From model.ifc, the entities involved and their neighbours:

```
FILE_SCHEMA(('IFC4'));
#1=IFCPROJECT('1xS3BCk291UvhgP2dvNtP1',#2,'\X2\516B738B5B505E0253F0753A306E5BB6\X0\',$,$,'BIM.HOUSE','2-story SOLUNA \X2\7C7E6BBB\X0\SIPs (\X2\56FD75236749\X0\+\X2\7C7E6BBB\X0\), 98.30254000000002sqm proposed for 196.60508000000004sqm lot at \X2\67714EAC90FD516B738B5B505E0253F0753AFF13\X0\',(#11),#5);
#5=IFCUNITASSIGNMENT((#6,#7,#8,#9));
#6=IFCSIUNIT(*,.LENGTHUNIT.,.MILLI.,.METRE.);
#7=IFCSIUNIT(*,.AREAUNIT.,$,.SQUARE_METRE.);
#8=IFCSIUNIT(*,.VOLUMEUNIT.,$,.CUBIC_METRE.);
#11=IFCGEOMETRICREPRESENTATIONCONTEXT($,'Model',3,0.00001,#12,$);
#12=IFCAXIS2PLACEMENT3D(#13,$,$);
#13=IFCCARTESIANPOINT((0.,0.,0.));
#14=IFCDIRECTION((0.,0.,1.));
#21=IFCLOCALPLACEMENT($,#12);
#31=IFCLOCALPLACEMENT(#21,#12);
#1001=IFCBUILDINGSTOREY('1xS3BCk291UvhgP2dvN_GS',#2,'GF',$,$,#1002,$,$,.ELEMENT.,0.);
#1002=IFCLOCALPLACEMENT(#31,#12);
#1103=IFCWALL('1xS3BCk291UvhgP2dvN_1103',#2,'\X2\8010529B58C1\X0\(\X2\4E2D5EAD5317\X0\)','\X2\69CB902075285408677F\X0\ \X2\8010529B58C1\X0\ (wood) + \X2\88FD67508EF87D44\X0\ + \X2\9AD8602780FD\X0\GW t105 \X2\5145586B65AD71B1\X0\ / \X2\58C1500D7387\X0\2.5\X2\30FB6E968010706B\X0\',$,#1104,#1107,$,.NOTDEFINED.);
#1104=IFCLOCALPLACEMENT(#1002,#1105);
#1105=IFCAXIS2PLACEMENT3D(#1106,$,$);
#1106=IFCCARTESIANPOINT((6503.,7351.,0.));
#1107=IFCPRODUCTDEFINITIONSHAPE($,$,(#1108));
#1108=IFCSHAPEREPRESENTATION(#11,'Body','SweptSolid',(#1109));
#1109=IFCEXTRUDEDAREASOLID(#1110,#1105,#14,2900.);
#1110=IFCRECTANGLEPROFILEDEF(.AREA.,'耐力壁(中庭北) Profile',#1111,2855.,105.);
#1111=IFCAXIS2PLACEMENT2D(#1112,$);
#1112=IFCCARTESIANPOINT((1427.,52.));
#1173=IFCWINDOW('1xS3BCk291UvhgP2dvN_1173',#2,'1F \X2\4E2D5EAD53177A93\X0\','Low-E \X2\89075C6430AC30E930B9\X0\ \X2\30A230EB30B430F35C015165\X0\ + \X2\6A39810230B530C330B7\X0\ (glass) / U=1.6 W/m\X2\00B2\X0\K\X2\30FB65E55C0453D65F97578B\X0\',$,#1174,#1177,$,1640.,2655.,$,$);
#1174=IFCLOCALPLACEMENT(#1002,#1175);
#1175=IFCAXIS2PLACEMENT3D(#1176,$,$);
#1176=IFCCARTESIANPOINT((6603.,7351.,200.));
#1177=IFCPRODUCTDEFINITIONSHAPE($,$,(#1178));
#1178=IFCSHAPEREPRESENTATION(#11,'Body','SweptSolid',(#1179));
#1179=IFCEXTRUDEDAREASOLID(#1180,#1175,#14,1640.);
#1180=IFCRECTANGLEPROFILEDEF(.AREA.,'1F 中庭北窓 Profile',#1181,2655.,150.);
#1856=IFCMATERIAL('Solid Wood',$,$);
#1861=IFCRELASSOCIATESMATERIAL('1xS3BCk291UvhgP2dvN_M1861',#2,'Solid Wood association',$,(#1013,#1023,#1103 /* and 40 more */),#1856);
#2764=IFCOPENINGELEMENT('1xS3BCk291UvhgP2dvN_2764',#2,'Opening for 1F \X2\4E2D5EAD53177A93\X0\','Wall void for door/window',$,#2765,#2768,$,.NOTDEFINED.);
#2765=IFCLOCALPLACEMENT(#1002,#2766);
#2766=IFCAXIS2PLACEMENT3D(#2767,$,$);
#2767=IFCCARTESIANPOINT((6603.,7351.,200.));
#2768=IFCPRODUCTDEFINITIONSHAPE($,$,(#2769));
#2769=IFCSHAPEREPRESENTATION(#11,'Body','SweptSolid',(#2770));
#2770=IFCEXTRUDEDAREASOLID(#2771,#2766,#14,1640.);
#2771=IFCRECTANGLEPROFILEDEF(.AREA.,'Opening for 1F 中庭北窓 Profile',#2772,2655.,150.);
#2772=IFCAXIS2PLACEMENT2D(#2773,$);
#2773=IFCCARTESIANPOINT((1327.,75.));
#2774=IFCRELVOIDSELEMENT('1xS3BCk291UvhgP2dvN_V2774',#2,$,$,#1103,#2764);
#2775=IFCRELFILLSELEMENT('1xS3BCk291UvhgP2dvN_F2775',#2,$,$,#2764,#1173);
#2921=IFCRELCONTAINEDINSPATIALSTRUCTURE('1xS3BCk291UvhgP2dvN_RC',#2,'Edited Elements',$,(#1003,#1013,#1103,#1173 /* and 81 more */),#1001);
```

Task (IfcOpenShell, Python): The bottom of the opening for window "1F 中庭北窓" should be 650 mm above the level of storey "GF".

```python
import numpy as np
import ifcopenshell
import ifcopenshell.api.geometry
import ifcopenshell.geom
import ifcopenshell.util.element
import ifcopenshell.util.placement
import ifcopenshell.util.shape
import ifcopenshell.util.unit

model = ifcopenshell.open("model.ifc")
unit_scale = ifcopenshell.util.unit.calculate_unit_scale(model)

window = model.by_guid("1xS3BCk291UvhgP2dvN_1173")
opening = window.FillsVoids[0].RelatingOpeningElement
storey = ifcopenshell.util.element.get_container(window, ifc_class="IfcBuildingStorey")
level = ifcopenshell.util.placement.get_local_placement(storey.ObjectPlacement)[2, 3]

# The opening's origin need not be at the sill, so measure its lowest point.
shape = ifcopenshell.geom.create_shape(ifcopenshell.geom.settings(), opening)
bottom = ifcopenshell.util.shape.get_shape_bottom_elevation(shape, shape.geometry) / unit_scale
dz = level + 650.0 - bottom

shift = np.array([0.0, 0.0, dz])
# The window is not placed relative to its opening, so move both.
for product in (opening, window):
    matrix = ifcopenshell.util.placement.get_local_placement(product.ObjectPlacement)
    matrix[:3, 3] += shift
    ifcopenshell.api.geometry.edit_object_placement(model, product=product, matrix=matrix, is_si=False)

print(f"moved by {dz * unit_scale:+.3f} m")

model.write("model_v2.ifc")
```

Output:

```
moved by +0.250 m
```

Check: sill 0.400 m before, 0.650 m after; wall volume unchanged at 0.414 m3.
